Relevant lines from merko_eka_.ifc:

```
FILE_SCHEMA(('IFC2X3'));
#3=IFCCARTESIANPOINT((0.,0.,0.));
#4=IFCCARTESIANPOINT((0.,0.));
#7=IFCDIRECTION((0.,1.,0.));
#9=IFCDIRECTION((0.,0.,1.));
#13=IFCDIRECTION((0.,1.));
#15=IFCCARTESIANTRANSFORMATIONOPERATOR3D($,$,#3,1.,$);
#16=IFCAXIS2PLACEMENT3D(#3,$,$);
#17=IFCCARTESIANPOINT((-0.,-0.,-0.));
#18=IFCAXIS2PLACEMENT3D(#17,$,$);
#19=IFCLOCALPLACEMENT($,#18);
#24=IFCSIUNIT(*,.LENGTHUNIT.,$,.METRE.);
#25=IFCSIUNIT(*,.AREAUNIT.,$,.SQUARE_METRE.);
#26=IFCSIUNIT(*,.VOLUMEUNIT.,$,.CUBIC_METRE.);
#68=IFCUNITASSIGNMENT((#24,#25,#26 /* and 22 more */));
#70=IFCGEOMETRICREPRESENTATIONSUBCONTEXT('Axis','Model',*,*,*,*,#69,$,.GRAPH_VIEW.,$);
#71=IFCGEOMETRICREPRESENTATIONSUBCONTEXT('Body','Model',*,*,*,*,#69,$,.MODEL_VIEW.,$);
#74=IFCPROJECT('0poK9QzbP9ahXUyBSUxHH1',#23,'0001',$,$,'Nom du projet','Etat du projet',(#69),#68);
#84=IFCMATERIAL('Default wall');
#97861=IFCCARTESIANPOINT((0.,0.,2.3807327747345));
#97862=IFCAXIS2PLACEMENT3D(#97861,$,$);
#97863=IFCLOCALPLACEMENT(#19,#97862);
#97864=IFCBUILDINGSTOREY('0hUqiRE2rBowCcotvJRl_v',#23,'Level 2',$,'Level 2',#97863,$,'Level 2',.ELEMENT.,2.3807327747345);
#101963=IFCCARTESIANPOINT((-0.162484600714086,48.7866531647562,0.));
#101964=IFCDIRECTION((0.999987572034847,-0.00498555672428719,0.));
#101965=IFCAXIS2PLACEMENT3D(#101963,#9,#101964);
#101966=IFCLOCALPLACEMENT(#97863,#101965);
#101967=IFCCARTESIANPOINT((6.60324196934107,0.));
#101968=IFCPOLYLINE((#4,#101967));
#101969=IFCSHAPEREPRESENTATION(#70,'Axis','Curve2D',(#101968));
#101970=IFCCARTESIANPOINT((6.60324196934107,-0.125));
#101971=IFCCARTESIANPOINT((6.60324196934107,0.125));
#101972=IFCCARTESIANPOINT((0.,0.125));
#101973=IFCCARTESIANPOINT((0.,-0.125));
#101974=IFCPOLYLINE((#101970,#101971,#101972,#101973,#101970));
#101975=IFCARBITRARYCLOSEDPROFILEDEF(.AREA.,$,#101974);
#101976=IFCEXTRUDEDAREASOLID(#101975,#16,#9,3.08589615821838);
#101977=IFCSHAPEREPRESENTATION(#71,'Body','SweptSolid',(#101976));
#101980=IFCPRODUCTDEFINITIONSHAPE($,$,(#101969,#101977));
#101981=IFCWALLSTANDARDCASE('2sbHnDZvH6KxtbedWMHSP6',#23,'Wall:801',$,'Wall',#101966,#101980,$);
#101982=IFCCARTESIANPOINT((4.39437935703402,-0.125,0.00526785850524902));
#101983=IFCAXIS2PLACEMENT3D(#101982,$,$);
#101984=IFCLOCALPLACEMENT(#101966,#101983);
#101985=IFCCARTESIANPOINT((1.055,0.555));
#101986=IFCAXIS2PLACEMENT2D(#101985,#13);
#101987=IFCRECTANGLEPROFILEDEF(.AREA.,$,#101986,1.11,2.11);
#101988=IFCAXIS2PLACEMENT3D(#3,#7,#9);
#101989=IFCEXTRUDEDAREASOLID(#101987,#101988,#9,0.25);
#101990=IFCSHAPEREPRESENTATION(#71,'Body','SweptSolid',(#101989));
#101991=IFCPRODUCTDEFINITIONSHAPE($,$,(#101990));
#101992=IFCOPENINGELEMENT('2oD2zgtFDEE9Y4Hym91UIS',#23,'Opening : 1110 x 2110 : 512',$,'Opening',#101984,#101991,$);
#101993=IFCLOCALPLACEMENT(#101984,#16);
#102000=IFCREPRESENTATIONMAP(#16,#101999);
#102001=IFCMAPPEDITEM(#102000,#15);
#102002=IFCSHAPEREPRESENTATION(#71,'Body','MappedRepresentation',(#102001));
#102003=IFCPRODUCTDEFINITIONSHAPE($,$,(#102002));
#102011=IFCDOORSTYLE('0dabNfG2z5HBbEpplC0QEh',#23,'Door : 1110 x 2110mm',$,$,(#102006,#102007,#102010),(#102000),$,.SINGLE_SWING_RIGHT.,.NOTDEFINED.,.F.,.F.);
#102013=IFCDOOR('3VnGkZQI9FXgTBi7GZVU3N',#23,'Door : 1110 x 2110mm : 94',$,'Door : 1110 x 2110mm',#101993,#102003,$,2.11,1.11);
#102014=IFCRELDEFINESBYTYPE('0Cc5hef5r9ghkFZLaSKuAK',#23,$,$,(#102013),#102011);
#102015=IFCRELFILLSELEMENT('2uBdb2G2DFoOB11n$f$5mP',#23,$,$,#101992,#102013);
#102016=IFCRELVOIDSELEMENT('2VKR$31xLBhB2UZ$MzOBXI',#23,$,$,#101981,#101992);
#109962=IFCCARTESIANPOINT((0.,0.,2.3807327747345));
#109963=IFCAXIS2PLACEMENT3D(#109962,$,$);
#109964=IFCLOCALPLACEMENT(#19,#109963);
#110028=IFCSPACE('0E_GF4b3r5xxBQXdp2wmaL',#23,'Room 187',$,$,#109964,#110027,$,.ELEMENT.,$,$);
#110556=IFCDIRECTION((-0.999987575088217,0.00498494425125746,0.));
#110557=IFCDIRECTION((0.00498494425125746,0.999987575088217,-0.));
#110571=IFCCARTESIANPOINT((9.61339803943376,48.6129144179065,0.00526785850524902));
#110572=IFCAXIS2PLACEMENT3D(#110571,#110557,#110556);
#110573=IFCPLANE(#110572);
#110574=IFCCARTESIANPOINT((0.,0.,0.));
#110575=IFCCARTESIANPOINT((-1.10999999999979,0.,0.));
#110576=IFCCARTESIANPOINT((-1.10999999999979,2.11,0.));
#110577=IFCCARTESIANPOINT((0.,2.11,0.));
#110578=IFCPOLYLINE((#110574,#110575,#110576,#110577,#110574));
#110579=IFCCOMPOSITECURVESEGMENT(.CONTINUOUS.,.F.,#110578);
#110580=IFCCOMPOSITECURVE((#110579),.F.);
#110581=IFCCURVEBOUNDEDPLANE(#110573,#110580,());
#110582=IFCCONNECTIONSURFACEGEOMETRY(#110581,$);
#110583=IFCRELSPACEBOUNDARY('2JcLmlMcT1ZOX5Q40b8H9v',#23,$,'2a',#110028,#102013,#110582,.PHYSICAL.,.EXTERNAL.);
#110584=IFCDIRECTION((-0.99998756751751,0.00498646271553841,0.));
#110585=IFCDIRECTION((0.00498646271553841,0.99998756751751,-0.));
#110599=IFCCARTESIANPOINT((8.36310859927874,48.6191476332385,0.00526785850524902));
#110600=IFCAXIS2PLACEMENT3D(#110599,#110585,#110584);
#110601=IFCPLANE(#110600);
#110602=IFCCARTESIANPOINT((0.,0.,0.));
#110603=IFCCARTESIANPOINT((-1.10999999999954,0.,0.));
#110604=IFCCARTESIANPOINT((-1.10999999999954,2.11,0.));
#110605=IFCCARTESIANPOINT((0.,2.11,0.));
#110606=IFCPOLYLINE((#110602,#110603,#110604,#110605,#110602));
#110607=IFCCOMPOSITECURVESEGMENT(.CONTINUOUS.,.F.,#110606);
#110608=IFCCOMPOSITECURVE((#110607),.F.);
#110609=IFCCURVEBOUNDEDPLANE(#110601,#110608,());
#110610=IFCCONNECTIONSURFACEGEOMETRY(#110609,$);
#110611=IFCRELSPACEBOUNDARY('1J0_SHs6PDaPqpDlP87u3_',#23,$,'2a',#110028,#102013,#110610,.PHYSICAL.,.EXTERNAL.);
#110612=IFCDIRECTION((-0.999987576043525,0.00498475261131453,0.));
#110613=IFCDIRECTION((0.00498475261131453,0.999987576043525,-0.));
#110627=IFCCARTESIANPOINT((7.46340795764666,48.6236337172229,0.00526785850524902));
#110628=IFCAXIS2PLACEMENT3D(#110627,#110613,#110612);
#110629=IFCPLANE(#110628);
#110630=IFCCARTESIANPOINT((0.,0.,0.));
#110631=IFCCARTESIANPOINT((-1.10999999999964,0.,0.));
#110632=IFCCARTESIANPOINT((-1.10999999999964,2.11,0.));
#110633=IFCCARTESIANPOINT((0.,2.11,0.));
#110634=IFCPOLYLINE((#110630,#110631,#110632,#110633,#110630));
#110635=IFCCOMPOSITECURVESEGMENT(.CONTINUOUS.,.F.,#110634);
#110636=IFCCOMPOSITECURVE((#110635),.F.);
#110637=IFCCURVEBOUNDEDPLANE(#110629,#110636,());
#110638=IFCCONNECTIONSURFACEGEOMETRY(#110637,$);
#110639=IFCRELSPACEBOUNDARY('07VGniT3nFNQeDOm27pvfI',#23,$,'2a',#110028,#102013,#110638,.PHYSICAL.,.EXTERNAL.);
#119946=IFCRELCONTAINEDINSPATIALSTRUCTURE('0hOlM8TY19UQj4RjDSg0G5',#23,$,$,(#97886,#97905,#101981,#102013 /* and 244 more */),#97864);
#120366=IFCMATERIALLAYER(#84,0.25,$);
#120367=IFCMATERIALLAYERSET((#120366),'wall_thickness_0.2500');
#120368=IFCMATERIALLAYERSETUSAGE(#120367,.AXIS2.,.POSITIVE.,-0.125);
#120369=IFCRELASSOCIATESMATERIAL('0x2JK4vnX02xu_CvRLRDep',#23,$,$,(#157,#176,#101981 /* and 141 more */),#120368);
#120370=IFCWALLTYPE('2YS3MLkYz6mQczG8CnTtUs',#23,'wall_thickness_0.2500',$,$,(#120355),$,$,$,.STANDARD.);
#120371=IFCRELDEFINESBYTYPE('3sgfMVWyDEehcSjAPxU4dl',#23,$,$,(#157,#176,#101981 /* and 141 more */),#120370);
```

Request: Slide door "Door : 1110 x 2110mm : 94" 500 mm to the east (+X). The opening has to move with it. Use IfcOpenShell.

```python
import numpy as np
import ifcopenshell
import ifcopenshell.api.geometry
import ifcopenshell.util.placement
import ifcopenshell.util.unit

model = ifcopenshell.open("merko_eka_.ifc")
unit_scale = ifcopenshell.util.unit.calculate_unit_scale(model)

door = model.by_id(102013)
opening = door.FillsVoids[0].RelatingOpeningElement
wall = opening.VoidsElements[0].RelatingBuildingElement

wall_matrix = ifcopenshell.util.placement.get_local_placement(wall.ObjectPlacement)
shift = wall_matrix[:3, 0] * 0.5 / unit_scale
before = ifcopenshell.util.placement.get_local_placement(door.ObjectPlacement)[:3, 3].copy()

# The door is placed relative to its opening, so it follows when the opening moves.
matrix = ifcopenshell.util.placement.get_local_placement(opening.ObjectPlacement)
matrix[:3, 3] += shift
ifcopenshell.api.geometry.edit_object_placement(
    model, product=opening, matrix=matrix, is_si=False, should_transform_children=True
)

# Space boundary surfaces are stored in each space's coordinates; move them too.
for rel in door.ProvidesBoundaries:
    if not rel.ConnectionGeometry:
        continue
    surface = rel.ConnectionGeometry.SurfaceOnRelatingElement.BasisSurface
    space_matrix = ifcopenshell.util.placement.get_local_placement(rel.RelatingSpace.ObjectPlacement)
    point = np.array(surface.Position.Location.Coordinates) + space_matrix[:3, :3].T @ shift
    surface.Position = model.createIfcAxis2Placement3D(
        model.createIfcCartesianPoint(point.tolist()), surface.Position.Axis, surface.Position.RefDirection
    )

after = ifcopenshell.util.placement.get_local_placement(door.ObjectPlacement)[:3, 3]
print("door moved by", (after - before).round(3) + 0.0)

model.write("merko_eka_-out.ifc")
```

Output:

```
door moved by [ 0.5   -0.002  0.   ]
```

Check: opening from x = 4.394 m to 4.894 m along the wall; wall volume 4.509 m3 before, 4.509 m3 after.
